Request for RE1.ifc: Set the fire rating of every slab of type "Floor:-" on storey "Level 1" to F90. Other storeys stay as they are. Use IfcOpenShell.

First a look at what the model holds.

```python
import ifcopenshell
import ifcopenshell.util.element

model = ifcopenshell.open("RE1.ifc")
print(model.schema)
storey = next(s for s in model.by_type("IfcBuildingStorey") if s.Name == "Level 1")
slabs = [e for e in ifcopenshell.util.element.get_decomposition(storey) if e.is_a("IfcSlab")]
seen = {}
for e in slabs:
    element_type = ifcopenshell.util.element.get_type(e)
    key = (element_type.Name if element_type != e and element_type else None, ifcopenshell.util.element.get_pset(e, "Pset_SlabCommon", "FireRating"))
    seen[key] = seen.get(key, 0) + 1
for (name, value), count in sorted(seen.items(), key=str):
    print(count, "x", name, "|", value)
```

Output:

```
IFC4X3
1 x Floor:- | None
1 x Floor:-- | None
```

```python
import ifcopenshell
import ifcopenshell.api.pset
import ifcopenshell.util.element

model = ifcopenshell.open("RE1.ifc")

storey = next(s for s in model.by_type("IfcBuildingStorey") if s.Name == "Level 1")
slabs = [e for e in ifcopenshell.util.element.get_decomposition(storey) if e.is_a("IfcSlab")]

count = 0
for e in slabs:
    element_type = ifcopenshell.util.element.get_type(e)
    if element_type in (None, e) or element_type.Name != "Floor:-":
        continue
    # add_pset returns the element's existing set when there is one.
    pset = ifcopenshell.api.pset.add_pset(model, product=e, name="Pset_SlabCommon")
    ifcopenshell.api.pset.edit_pset(model, pset=pset, properties={"FireRating": "F90"})
    count += 1

print(count, "slabs updated")

model.write("RE1-out.ifc")
```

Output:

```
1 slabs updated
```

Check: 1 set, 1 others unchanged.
